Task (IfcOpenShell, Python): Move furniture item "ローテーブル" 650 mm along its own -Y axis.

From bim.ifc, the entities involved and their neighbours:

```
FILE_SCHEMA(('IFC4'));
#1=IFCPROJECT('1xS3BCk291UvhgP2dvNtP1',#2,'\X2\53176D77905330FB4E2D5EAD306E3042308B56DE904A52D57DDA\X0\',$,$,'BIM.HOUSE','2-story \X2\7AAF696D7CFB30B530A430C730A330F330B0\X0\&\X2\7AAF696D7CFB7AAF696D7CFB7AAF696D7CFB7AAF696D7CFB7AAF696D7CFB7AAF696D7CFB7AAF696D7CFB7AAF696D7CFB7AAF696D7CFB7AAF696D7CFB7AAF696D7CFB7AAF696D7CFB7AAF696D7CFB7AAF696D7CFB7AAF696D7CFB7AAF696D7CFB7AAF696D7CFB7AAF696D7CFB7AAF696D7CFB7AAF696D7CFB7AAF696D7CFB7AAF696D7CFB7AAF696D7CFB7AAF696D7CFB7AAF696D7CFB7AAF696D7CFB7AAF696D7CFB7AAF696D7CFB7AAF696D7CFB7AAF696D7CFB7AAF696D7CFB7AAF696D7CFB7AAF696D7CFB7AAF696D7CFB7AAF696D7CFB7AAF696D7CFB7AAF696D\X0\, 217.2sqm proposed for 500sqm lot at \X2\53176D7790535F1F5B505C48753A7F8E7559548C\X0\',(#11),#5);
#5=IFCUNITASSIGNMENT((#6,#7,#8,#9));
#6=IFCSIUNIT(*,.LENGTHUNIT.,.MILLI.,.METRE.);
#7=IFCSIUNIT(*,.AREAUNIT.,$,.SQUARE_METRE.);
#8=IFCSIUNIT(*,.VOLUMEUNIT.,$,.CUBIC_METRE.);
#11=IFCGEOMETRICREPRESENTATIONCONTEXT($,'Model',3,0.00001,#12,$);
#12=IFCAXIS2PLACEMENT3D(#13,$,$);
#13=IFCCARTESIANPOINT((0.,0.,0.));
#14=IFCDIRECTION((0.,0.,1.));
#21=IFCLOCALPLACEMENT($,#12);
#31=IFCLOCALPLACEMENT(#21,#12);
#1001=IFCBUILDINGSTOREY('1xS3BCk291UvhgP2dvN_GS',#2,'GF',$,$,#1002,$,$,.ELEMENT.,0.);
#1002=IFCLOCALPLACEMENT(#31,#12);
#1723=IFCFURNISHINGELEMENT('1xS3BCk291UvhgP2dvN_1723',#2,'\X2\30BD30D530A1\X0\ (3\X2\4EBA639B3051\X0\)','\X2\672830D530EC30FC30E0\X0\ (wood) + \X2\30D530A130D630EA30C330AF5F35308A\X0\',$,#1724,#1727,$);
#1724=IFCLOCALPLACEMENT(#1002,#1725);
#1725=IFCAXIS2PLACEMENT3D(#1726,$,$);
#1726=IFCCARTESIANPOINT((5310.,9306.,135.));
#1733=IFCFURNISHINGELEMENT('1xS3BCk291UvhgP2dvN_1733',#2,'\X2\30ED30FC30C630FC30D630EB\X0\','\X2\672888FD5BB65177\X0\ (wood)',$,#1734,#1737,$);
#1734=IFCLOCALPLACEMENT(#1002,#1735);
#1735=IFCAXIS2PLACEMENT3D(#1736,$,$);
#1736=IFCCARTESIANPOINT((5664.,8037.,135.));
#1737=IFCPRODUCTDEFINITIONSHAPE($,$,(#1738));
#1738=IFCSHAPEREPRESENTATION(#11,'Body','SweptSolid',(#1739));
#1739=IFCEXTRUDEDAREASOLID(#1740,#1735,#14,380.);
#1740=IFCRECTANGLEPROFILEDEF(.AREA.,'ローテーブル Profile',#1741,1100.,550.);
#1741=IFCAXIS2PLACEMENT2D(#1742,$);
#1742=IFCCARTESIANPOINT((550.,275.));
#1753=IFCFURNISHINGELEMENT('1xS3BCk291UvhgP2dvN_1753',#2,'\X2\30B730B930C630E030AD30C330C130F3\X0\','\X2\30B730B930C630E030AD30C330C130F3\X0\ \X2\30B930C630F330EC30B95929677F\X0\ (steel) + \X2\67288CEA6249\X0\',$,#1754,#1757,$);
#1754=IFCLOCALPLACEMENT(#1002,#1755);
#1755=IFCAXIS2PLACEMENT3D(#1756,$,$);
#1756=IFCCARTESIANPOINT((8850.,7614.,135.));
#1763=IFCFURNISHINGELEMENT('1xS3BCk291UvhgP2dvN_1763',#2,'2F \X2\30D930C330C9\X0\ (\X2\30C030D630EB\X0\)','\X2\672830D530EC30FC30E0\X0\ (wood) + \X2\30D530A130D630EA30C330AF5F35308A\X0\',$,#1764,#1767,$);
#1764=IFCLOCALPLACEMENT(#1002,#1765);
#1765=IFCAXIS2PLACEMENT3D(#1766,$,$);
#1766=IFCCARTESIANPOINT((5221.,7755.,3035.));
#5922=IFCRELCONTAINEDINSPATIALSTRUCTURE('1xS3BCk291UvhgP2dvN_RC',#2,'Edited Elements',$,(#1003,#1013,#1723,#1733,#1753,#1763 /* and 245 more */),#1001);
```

```python
import ifcopenshell
import ifcopenshell.api.geometry
import ifcopenshell.util.placement
import ifcopenshell.util.unit

model = ifcopenshell.open("bim.ifc")
unit_scale = ifcopenshell.util.unit.calculate_unit_scale(model)

item = model.by_guid("1xS3BCk291UvhgP2dvN_1733")
matrix = ifcopenshell.util.placement.get_local_placement(item.ObjectPlacement)
matrix[:3, 3] -= matrix[:3, 1] * 0.65 / unit_scale
ifcopenshell.api.geometry.edit_object_placement(model, product=item, matrix=matrix, is_si=False)

print(ifcopenshell.util.placement.get_local_placement(item.ObjectPlacement).round(3) + 0.0)

model.write("bim-out.ifc")
```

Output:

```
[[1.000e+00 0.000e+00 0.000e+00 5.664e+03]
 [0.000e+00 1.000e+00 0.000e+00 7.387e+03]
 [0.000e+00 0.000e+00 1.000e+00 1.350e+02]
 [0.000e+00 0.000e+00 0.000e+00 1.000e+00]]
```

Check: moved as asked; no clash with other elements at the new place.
